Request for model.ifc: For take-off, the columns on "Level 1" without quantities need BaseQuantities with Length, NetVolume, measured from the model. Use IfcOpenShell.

First a look at what the model holds.

```python
import ifcopenshell
import ifcopenshell.util.element
import ifcopenshell.util.unit

model = ifcopenshell.open("model.ifc")
print(model.schema)
for unit_type in ("LENGTHUNIT", "AREAUNIT", "VOLUMEUNIT"):
    print(unit_type, ifcopenshell.util.unit.calculate_unit_scale(model, unit_type))
storey = next(s for s in model.by_type("IfcBuildingStorey") if s.Name == "Level 1")
columns = [e for e in ifcopenshell.util.element.get_decomposition(storey) if e.is_a("IfcColumn")]
for e in sorted(columns, key=lambda e: e.id()):
    print(e.id(), e.is_a(), e.Name, list(ifcopenshell.util.element.get_psets(e, qtos_only=True)), sep=" | ")
```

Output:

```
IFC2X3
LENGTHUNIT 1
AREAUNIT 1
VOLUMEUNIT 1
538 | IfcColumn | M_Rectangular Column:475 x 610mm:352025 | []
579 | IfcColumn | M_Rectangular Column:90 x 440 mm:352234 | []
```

```python
import ifcopenshell
import ifcopenshell.api.pset
import ifcopenshell.geom
import ifcopenshell.util.element
import ifcopenshell.util.shape
import ifcopenshell.util.unit

model = ifcopenshell.open("model.ifc")
unit_scale = ifcopenshell.util.unit.calculate_unit_scale(model)
volume_scale = ifcopenshell.util.unit.calculate_unit_scale(model, "VOLUMEUNIT")
settings = ifcopenshell.geom.settings()

storey = next(s for s in model.by_type("IfcBuildingStorey") if s.Name == "Level 1")
columns = [e for e in ifcopenshell.util.element.get_decomposition(storey) if e.is_a("IfcColumn")]

for e in sorted(columns, key=lambda e: e.id()):
    if ifcopenshell.util.element.get_psets(e, qtos_only=True, should_inherit=False):
        continue
    # Geometry comes back in metres, in the element's own axes.
    shape = ifcopenshell.geom.create_shape(settings, e)
    values = {
        "Length": ifcopenshell.util.shape.get_z(shape.geometry) / unit_scale,
        "NetVolume": ifcopenshell.util.shape.get_volume(shape.geometry) / volume_scale,
    }
    qto = ifcopenshell.api.pset.add_qto(model, product=e, name="BaseQuantities")
    ifcopenshell.api.pset.edit_qto(model, qto=qto, properties=values)
    print(e.id(), {k: round(v, 3) for k, v in values.items()})

model.write("model_edited.ifc")
```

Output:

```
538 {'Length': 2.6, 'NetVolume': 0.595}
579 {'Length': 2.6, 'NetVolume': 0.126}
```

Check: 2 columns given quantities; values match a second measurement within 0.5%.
